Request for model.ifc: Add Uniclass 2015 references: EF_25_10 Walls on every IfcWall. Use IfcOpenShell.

First a look at what the model holds.

```python
import ifcopenshell

model = ifcopenshell.open("model.ifc")
print(model.schema)
print("classifications:", [c.Name for c in model.by_type("IfcClassification")])
for ifc_class in ("IfcDoor", "IfcRoof", "IfcStair", "IfcWall", "IfcWindow"):
    print(ifc_class, len(model.by_type(ifc_class)))
```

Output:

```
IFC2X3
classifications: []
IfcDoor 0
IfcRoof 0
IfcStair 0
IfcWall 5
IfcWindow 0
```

```python
import ifcopenshell
import ifcopenshell.api.classification

model = ifcopenshell.open("model.ifc")

# IFC2X3 requires Source and Edition and has no link from the project to the system.
system = model.create_entity("IfcClassification", Source="NBS", Edition="2015", Name="Uniclass 2015")

codes = {
    "IfcWall": ("EF_25_10", "Walls"),
}
for ifc_class, (code, name) in codes.items():
    products = model.by_type(ifc_class)
    ifcopenshell.api.classification.add_reference(
        model, products=products, classification=system, identification=code, name=name
    )
    print(code, len(products))

model.write("model_rev.ifc")
```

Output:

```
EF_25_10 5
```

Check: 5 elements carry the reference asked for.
